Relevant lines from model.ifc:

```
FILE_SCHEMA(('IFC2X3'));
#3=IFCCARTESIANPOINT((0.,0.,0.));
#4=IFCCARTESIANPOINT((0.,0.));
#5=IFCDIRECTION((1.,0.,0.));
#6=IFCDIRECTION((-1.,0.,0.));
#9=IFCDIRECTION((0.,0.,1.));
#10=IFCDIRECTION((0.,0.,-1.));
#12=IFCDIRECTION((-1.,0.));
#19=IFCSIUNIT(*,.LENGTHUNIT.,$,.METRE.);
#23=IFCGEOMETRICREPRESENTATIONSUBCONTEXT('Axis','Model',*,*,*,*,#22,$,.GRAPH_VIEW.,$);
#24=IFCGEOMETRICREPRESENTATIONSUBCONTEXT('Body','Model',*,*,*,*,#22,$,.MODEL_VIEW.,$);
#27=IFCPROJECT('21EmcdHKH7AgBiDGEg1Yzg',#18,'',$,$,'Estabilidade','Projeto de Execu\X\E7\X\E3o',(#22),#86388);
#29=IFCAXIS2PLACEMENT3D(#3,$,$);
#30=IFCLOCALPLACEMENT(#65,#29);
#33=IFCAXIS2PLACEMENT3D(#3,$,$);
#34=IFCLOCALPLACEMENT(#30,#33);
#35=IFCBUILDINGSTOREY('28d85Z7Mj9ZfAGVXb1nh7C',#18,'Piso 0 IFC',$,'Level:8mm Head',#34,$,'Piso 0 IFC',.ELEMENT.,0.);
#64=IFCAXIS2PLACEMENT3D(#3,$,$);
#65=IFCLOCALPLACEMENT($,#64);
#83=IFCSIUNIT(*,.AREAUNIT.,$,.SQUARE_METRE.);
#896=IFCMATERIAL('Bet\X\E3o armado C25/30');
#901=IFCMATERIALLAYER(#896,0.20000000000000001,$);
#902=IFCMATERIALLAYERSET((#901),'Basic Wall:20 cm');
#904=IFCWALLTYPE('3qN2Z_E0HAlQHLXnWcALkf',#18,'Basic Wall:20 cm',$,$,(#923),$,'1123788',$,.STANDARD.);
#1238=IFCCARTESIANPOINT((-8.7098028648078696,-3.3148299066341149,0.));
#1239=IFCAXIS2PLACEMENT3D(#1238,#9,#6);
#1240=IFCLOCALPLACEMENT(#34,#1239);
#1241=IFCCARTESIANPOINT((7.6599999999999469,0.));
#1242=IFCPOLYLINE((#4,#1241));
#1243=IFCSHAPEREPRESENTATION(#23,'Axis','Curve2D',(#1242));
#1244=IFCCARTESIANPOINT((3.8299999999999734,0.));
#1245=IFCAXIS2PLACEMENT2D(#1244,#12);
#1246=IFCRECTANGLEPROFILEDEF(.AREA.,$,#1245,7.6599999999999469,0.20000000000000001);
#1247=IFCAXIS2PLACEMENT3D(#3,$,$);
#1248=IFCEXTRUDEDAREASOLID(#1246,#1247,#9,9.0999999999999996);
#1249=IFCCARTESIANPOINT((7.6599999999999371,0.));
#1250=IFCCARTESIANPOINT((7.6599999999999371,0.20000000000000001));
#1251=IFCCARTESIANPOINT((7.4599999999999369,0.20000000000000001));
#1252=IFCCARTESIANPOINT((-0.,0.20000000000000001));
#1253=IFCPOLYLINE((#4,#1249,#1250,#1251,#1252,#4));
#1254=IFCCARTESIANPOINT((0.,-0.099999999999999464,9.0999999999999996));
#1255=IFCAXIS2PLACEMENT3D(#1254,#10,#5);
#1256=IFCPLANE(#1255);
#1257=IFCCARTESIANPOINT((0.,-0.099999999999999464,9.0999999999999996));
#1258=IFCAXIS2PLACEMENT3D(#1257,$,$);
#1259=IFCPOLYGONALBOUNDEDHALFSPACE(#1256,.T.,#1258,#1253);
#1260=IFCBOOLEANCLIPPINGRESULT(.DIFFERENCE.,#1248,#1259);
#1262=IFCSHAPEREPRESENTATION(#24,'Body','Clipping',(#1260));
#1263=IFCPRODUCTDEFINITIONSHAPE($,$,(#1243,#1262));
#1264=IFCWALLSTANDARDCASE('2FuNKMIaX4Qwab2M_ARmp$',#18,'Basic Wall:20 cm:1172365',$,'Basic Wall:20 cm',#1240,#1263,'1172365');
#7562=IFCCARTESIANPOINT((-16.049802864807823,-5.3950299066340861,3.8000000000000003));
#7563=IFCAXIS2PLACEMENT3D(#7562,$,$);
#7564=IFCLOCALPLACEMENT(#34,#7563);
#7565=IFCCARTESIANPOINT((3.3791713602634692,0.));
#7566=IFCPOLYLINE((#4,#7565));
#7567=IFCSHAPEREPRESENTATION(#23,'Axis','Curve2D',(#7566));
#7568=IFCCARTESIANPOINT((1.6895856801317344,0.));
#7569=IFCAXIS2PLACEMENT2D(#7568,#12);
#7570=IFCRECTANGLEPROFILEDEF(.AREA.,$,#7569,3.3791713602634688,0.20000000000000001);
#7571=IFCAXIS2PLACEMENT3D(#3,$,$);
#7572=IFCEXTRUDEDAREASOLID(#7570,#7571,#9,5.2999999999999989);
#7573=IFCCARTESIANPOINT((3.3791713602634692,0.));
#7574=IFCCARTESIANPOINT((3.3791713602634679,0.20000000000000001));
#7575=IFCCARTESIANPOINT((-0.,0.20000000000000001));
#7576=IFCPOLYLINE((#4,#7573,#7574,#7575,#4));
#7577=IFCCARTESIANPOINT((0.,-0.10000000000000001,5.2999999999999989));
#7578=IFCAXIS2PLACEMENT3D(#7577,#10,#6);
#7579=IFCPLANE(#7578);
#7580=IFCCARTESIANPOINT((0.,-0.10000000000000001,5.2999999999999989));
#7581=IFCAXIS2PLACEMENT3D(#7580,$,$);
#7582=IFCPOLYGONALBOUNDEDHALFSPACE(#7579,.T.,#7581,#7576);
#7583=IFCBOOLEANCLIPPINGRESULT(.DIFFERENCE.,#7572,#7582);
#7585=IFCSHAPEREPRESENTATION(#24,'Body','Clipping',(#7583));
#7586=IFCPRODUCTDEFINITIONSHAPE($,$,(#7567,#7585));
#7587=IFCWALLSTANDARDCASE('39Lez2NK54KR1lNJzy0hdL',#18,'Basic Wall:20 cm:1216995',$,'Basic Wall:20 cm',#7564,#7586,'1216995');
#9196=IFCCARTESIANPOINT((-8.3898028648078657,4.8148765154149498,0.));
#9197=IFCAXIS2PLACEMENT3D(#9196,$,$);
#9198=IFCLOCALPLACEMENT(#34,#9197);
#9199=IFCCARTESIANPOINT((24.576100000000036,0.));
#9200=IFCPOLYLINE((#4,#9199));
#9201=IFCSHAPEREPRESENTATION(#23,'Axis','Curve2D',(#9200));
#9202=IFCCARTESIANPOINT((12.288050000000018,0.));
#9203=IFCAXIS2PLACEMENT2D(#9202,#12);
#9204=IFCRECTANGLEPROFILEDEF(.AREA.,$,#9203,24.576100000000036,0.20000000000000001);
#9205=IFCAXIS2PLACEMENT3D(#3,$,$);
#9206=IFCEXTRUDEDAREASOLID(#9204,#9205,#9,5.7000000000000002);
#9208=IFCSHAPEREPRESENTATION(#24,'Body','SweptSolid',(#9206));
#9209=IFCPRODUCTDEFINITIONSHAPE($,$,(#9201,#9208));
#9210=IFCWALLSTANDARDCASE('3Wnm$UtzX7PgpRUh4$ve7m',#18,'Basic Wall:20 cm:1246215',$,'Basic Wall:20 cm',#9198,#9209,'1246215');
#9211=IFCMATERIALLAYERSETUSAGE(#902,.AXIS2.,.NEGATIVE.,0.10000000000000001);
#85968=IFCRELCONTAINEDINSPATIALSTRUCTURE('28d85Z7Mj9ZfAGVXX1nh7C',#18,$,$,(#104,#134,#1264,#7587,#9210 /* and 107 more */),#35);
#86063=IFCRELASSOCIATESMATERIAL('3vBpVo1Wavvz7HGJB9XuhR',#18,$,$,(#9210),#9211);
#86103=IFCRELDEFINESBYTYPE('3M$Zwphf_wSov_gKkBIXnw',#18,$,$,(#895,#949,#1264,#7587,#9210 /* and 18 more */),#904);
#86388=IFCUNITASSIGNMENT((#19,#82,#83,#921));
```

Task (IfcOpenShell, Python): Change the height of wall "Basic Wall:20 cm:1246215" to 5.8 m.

```python
import ifcopenshell
import ifcopenshell.geom
import ifcopenshell.util.representation
import ifcopenshell.util.shape
import ifcopenshell.util.unit

model = ifcopenshell.open("model.ifc")
unit_scale = ifcopenshell.util.unit.calculate_unit_scale(model)
settings = ifcopenshell.geom.settings()


def volume(element):
    """Net volume in cubic metres, openings subtracted."""
    shape = ifcopenshell.geom.create_shape(settings, element)
    return ifcopenshell.util.shape.get_volume(shape.geometry)


wall = model.by_id(9210)
before = volume(wall)

body = ifcopenshell.util.representation.get_representation(wall, "Model", "Body")
solid = body.Items[0]
old_height = solid.Depth
solid.Depth = 5.8 / unit_scale
after = volume(wall)

print(f"height {old_height:g} -> {solid.Depth:g}, volume {before:.3f} -> {after:.3f} m3")

model.write("model_edited.ifc")
```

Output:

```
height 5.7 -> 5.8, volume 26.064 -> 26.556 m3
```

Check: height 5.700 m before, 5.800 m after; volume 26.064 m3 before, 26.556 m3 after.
